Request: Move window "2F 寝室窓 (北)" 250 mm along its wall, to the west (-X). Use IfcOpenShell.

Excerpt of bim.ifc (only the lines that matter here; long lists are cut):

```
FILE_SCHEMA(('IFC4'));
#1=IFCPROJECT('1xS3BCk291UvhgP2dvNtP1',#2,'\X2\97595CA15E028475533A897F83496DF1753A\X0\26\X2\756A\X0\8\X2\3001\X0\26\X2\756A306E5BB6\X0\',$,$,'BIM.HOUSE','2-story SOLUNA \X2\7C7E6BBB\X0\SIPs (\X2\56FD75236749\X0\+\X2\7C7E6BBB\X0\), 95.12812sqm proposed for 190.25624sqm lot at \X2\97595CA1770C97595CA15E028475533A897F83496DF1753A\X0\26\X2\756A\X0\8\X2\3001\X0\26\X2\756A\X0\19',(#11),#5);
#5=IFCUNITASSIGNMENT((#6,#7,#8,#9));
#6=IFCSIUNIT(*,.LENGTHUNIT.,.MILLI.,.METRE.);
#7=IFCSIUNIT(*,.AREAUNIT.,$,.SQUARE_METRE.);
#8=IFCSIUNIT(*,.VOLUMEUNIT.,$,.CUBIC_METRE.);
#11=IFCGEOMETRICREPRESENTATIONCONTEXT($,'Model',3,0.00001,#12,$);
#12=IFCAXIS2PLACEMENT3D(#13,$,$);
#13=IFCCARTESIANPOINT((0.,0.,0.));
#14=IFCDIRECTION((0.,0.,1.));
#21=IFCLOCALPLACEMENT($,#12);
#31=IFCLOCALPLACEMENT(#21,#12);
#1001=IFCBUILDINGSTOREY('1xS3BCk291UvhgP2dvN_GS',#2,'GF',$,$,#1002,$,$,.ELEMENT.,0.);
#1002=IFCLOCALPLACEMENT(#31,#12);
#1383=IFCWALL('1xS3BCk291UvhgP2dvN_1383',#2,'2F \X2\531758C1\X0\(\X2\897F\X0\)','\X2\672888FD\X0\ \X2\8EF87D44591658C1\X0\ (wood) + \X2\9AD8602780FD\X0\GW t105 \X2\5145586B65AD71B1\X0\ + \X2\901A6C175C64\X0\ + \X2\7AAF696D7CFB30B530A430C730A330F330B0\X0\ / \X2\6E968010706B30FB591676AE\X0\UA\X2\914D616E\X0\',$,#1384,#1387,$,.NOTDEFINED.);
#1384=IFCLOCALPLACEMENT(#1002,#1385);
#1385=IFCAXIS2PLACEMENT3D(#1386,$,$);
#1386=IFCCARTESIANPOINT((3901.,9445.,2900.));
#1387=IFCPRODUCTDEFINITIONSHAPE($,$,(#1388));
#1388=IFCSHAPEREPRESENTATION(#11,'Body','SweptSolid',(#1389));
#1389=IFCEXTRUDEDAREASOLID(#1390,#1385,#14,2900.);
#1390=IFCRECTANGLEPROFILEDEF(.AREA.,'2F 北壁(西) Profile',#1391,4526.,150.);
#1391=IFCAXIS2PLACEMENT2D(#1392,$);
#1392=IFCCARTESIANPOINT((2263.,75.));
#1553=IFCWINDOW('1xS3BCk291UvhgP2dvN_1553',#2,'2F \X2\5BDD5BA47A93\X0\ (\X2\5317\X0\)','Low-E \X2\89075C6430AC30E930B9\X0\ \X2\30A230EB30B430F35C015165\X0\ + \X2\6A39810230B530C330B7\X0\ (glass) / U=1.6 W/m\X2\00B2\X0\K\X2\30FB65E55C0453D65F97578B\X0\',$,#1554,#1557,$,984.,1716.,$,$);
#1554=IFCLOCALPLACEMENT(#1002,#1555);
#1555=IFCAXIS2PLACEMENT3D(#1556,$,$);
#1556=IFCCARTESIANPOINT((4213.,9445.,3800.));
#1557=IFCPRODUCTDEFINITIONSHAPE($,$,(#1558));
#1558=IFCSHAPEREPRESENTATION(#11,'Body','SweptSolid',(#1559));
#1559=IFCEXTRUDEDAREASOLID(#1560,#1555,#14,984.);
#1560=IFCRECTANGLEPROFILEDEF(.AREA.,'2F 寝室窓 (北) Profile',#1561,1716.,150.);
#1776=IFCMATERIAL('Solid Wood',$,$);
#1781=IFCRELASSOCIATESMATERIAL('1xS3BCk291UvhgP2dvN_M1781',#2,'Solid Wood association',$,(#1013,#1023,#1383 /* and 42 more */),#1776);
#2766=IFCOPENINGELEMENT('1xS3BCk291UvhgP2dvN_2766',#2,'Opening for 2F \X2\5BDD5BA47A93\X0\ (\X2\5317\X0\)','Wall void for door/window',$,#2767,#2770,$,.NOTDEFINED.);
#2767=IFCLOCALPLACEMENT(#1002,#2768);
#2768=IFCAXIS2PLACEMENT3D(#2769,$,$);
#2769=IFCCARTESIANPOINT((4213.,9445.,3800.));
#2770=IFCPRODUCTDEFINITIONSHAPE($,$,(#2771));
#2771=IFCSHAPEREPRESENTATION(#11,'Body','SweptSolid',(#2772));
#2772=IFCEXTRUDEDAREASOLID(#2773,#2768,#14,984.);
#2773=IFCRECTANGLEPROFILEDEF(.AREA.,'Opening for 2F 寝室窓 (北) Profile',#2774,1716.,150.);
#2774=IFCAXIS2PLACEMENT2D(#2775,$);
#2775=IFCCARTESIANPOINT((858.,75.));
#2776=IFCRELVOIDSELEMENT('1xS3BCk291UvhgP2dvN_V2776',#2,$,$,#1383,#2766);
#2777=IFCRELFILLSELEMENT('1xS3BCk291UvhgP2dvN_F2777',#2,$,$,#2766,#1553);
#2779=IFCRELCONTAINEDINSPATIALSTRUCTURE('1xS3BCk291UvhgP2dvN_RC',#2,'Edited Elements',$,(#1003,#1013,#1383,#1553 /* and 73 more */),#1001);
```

```python
import ifcopenshell
import ifcopenshell.api.geometry
import ifcopenshell.util.placement
import ifcopenshell.util.unit

model = ifcopenshell.open("bim.ifc")
unit_scale = ifcopenshell.util.unit.calculate_unit_scale(model)

window = model.by_guid("1xS3BCk291UvhgP2dvN_1553")
opening = window.FillsVoids[0].RelatingOpeningElement
wall = opening.VoidsElements[0].RelatingBuildingElement

wall_matrix = ifcopenshell.util.placement.get_local_placement(wall.ObjectPlacement)
shift = wall_matrix[:3, 0] * -0.25 / unit_scale
before = ifcopenshell.util.placement.get_local_placement(window.ObjectPlacement)[:3, 3].copy()

# The window is not placed relative to its opening, so move both.
for product in (opening, window):
    matrix = ifcopenshell.util.placement.get_local_placement(product.ObjectPlacement)
    matrix[:3, 3] += shift
    ifcopenshell.api.geometry.edit_object_placement(model, product=product, matrix=matrix, is_si=False)

after = ifcopenshell.util.placement.get_local_placement(window.ObjectPlacement)[:3, 3]
print("window moved by", (after - before).round(3) + 0.0)

model.write("bim_rev.ifc")
```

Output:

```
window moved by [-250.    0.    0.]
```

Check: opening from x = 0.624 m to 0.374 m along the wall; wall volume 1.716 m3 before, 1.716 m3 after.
